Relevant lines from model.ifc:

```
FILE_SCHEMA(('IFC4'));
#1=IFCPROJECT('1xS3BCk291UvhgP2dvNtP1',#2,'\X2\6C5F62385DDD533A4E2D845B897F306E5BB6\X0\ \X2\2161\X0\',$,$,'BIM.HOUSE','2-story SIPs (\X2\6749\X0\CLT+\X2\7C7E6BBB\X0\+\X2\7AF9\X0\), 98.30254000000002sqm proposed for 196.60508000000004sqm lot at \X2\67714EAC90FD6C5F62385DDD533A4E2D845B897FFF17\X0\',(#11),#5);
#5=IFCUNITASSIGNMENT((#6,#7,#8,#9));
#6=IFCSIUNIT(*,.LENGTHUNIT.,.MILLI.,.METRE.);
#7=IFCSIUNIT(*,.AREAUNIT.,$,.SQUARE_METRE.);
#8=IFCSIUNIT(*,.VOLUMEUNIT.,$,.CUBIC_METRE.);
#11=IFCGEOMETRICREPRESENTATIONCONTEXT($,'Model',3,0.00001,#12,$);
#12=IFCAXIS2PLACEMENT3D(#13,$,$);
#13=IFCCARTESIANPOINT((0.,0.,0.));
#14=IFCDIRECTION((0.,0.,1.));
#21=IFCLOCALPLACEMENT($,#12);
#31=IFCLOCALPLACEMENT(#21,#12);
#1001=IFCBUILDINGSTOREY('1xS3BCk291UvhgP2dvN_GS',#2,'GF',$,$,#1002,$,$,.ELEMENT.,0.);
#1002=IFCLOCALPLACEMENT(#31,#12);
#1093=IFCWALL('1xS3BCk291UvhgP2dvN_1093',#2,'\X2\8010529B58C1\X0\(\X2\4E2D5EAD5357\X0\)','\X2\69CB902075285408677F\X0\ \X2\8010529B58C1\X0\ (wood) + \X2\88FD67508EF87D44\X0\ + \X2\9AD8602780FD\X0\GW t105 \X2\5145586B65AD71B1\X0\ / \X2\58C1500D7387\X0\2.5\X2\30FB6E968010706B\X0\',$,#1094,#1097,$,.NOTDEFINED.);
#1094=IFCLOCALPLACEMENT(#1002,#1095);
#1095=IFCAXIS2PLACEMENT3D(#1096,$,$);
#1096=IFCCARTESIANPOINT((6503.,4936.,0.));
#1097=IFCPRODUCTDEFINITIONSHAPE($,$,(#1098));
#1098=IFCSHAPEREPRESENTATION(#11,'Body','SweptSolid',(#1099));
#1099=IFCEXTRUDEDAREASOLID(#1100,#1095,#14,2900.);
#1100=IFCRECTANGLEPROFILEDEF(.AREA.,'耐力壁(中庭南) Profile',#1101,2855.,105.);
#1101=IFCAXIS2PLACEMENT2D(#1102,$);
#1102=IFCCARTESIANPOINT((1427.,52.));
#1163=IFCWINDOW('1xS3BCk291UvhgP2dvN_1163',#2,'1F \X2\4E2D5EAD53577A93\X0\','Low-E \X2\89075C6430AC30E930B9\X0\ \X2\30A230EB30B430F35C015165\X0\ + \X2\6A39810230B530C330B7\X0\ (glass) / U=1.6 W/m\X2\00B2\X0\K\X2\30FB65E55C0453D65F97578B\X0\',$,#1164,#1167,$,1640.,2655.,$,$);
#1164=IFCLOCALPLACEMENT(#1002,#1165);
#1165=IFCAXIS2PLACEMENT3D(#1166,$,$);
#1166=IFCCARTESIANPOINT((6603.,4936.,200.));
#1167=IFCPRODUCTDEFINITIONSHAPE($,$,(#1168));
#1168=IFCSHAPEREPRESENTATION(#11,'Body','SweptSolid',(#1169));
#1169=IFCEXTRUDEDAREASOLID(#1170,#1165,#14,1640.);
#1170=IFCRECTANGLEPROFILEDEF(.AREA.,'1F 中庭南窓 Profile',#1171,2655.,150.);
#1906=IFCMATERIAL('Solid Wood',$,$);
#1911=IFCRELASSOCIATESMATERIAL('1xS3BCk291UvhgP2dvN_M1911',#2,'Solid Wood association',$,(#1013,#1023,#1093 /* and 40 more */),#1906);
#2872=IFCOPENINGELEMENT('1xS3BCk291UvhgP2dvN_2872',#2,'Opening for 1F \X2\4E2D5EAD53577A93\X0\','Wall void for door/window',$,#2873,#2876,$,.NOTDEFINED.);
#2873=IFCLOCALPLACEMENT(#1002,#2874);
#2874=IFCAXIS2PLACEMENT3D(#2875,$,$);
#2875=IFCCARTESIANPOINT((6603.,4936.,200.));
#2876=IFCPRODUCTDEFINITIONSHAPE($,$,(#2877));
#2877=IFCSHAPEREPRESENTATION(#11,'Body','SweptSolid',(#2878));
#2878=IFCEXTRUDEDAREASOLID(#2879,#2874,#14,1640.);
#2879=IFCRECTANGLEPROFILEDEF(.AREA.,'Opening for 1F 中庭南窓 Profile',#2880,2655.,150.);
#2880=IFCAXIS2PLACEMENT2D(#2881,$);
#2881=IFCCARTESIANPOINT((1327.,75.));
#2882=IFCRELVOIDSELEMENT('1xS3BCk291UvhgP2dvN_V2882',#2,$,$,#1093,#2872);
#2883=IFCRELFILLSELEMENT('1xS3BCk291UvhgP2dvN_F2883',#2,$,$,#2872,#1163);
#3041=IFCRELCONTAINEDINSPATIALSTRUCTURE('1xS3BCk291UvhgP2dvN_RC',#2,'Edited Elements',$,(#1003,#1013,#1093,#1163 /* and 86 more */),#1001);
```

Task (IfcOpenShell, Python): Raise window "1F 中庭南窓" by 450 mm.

```python
import numpy as np
import ifcopenshell
import ifcopenshell.api.geometry
import ifcopenshell.util.placement
import ifcopenshell.util.unit

model = ifcopenshell.open("model.ifc")
unit_scale = ifcopenshell.util.unit.calculate_unit_scale(model)

window = model.by_guid("1xS3BCk291UvhgP2dvN_1163")
opening = window.FillsVoids[0].RelatingOpeningElement
dz = 0.45 / unit_scale

shift = np.array([0.0, 0.0, dz])
# The window is not placed relative to its opening, so move both.
for product in (opening, window):
    matrix = ifcopenshell.util.placement.get_local_placement(product.ObjectPlacement)
    matrix[:3, 3] += shift
    ifcopenshell.api.geometry.edit_object_placement(model, product=product, matrix=matrix, is_si=False)

print(f"moved by {dz * unit_scale:+.3f} m")

model.write("model_updated.ifc")
```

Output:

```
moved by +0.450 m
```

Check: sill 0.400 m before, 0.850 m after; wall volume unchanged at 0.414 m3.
